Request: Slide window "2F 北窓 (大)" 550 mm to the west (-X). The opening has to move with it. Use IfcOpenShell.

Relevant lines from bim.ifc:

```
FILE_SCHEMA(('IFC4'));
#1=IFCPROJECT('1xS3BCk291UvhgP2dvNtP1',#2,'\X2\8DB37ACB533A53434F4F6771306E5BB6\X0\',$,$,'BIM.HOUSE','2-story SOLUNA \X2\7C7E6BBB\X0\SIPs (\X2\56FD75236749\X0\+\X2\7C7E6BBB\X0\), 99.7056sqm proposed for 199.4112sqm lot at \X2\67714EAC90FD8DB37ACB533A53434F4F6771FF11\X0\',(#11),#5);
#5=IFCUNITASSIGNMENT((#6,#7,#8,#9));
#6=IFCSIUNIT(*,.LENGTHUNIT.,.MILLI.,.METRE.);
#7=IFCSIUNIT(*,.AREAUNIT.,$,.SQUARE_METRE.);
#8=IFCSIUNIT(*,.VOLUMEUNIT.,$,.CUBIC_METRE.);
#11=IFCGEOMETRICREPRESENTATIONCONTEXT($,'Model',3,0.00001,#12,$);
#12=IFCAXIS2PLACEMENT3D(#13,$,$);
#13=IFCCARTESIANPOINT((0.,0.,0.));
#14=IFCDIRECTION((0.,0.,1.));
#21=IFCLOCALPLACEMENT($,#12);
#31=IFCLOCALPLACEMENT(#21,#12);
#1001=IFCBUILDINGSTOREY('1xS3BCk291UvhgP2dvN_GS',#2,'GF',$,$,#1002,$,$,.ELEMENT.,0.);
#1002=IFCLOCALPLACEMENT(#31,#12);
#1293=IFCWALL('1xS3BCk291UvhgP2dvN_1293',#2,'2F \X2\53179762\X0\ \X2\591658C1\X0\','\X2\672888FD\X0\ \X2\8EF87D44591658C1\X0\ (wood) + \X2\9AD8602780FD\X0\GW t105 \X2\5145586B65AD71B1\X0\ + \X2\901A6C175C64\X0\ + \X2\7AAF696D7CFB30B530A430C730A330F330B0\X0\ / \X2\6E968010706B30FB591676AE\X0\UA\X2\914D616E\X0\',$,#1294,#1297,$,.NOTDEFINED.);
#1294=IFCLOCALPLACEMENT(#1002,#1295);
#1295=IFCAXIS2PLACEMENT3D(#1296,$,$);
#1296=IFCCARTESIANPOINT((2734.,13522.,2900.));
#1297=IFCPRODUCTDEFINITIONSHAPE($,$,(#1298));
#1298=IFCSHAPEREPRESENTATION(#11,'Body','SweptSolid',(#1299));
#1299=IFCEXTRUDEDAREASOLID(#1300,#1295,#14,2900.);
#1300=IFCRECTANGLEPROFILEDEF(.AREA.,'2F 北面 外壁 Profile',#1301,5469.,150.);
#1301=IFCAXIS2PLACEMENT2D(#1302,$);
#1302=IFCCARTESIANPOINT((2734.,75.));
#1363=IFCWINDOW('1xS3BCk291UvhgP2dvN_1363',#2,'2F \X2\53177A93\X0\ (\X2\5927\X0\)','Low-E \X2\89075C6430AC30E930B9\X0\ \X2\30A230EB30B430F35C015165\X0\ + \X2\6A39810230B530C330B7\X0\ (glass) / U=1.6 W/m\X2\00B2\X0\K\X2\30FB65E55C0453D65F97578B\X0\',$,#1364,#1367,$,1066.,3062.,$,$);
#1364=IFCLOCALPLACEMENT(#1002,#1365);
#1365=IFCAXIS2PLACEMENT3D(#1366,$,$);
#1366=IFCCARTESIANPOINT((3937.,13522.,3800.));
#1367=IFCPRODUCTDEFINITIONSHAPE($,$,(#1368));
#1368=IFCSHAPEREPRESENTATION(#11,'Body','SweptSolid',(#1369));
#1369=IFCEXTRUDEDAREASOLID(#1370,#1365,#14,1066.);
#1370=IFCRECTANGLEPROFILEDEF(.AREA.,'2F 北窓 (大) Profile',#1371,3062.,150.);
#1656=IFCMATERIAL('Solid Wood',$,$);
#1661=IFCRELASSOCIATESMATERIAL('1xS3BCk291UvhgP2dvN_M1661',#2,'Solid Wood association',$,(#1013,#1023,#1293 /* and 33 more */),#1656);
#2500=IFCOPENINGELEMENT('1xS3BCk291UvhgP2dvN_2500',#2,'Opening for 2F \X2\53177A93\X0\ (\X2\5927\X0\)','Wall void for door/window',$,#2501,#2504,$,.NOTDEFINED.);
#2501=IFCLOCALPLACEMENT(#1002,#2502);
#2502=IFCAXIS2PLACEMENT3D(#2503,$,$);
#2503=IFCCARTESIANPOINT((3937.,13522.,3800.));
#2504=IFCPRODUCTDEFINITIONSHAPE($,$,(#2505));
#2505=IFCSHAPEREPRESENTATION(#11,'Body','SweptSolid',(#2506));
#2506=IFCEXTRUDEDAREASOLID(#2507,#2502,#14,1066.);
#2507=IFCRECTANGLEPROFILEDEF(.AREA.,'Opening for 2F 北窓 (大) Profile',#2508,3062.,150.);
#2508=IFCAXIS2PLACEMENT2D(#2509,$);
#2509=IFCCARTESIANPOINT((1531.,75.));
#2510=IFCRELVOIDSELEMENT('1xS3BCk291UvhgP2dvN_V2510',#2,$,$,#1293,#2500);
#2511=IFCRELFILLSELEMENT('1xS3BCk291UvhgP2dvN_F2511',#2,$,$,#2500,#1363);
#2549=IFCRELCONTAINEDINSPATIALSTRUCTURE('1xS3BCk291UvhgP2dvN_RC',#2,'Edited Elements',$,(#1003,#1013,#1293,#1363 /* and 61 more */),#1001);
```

```python
import ifcopenshell
import ifcopenshell.api.geometry
import ifcopenshell.util.placement

model = ifcopenshell.open("bim.ifc")

window = model.by_guid("1xS3BCk291UvhgP2dvN_1363")
opening = window.FillsVoids[0].RelatingOpeningElement
wall = opening.VoidsElements[0].RelatingBuildingElement

wall_matrix = ifcopenshell.util.placement.get_local_placement(wall.ObjectPlacement)
shift = wall_matrix[:3, 0] * -550.0
before = ifcopenshell.util.placement.get_local_placement(window.ObjectPlacement)[:3, 3].copy()

# The window is not placed relative to its opening, so move both.
for product in (opening, window):
    matrix = ifcopenshell.util.placement.get_local_placement(product.ObjectPlacement)
    matrix[:3, 3] += shift
    ifcopenshell.api.geometry.edit_object_placement(model, product=product, matrix=matrix, is_si=False)

after = ifcopenshell.util.placement.get_local_placement(window.ObjectPlacement)[:3, 3]
print("window moved by", (after - before).round(3) + 0.0)

model.write("bim_edited.ifc")
```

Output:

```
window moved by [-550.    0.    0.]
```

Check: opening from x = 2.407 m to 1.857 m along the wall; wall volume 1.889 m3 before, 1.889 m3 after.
